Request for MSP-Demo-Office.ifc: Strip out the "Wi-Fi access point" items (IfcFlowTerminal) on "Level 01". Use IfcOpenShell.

First a look at what the model holds.

```python
import ifcopenshell
import ifcopenshell.util.element

model = ifcopenshell.open("MSP-Demo-Office.ifc")
print(model.schema)
storey = next(s for s in model.by_type("IfcBuildingStorey") if s.Name == "Level 01")
terminals = [e for e in ifcopenshell.util.element.get_decomposition(storey) if e.is_a("IfcFlowTerminal")]
seen = {}
for e in terminals:
    element_type = ifcopenshell.util.element.get_type(e)
    name = element_type.Name if element_type not in (None, e) else None
    seen[name] = seen.get(name, 0) + 1
for name, count in sorted(seen.items(), key=str):
    print(count, "x", name)
```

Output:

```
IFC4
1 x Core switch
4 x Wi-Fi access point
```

```python
import ifcopenshell
import ifcopenshell.api.root
import ifcopenshell.util.element

model = ifcopenshell.open("MSP-Demo-Office.ifc")

storey = next(s for s in model.by_type("IfcBuildingStorey") if s.Name == "Level 01")
terminals = [e for e in ifcopenshell.util.element.get_decomposition(storey) if e.is_a("IfcFlowTerminal")]
targets = [e for e in terminals if (t := ifcopenshell.util.element.get_type(e)) not in (None, e) and t.Name == "Wi-Fi access point"]

for e in targets:
    ifcopenshell.api.root.remove_product(model, product=e)
print(len(targets), "removed")

model.write("MSP-Demo-Office_rev.ifc")
```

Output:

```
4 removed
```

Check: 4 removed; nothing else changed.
